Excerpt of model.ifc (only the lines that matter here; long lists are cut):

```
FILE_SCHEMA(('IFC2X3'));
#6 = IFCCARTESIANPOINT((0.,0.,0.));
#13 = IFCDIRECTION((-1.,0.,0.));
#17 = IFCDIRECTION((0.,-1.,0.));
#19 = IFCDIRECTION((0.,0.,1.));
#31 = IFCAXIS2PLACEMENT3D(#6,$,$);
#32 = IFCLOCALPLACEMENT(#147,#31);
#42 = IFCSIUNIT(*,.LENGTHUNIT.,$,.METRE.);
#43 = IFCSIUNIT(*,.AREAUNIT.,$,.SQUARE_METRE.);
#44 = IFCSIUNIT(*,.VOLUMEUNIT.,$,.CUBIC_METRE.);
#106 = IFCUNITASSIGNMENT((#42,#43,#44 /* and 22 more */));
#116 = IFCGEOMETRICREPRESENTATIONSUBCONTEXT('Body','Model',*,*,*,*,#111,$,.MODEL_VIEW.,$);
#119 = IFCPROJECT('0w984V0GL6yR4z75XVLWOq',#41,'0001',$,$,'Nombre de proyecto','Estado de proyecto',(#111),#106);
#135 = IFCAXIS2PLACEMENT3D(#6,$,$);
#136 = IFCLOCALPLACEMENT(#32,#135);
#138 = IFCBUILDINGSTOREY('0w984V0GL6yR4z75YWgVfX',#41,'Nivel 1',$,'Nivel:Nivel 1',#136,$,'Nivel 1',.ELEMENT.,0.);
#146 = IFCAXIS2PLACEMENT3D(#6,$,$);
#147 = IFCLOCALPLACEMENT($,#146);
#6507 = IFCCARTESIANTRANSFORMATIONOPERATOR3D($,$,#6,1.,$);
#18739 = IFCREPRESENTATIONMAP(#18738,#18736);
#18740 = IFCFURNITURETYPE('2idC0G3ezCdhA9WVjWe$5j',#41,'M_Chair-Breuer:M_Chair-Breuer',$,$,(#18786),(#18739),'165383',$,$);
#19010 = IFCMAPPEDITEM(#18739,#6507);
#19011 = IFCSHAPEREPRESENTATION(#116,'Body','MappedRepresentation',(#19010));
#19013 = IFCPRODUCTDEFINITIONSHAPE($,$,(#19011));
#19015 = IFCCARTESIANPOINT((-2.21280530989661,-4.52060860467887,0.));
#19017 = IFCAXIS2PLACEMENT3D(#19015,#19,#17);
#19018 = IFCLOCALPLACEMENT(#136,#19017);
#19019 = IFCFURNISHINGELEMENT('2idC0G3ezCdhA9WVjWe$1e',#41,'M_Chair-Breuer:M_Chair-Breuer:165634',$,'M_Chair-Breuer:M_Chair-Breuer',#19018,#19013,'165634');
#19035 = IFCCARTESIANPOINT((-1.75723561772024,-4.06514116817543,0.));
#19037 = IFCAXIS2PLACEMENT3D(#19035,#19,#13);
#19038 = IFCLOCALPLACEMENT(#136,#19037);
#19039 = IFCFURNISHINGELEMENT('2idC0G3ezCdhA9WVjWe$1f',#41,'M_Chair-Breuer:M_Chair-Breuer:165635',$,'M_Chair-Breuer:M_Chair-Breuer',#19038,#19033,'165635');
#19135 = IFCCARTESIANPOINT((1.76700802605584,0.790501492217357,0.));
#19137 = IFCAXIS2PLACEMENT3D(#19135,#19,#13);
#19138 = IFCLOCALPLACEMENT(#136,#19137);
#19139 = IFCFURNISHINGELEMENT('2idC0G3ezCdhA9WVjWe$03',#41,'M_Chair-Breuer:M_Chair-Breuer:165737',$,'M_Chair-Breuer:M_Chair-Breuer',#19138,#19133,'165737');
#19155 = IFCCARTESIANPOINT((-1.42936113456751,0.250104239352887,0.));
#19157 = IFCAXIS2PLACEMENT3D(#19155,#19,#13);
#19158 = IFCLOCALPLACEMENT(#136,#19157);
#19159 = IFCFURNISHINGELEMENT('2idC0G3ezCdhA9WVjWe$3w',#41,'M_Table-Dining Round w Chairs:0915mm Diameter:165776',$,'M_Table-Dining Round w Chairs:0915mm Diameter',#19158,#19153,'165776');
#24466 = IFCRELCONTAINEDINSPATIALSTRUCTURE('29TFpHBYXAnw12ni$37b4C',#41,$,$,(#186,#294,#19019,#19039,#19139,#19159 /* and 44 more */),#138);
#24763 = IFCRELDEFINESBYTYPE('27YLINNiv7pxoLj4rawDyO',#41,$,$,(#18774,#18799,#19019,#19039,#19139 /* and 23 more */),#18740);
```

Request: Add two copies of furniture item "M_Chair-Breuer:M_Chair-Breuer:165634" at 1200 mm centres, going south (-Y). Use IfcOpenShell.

```python
import numpy as np
import ifcopenshell
import ifcopenshell.api.geometry
import ifcopenshell.api.root
import ifcopenshell.util.element
import ifcopenshell.util.placement

model = ifcopenshell.open("model.ifc")


def reuse_history(source, copy):
    """copy_class also copies each property set's owner history, people and application; keep the originals."""
    for rel in copy.IsDefinedBy:
        if rel.is_a("IfcRelDefinesByProperties") and (history := rel.RelatingPropertyDefinition.OwnerHistory):
            rel.RelatingPropertyDefinition.OwnerHistory = source.OwnerHistory
            ifcopenshell.util.element.remove_deep2(model, history)


source = model.by_guid("2idC0G3ezCdhA9WVjWe$1e")
base = ifcopenshell.util.placement.get_local_placement(source.ObjectPlacement)
step = np.array([0.0, -1.0, 0.0]) * 1.2

for i in range(1, 3):
    copy = ifcopenshell.api.root.copy_class(model, product=source)
    copy.Representation = ifcopenshell.util.element.copy_deep(
        model, source.Representation, exclude=["IfcGeometricRepresentationContext", "IfcRepresentationMap"]
    )
    copy.Name = "M_Chair-Breuer:M_Chair-Breuer"
    copy.Tag = None
    reuse_history(source, copy)
    matrix = base.copy()
    matrix[:3, 3] += i * step
    print("added at", matrix[:3, 3].round(3) + 0.0)
    ifcopenshell.api.geometry.edit_object_placement(model, product=copy, matrix=matrix, is_si=False)

model.write("model_rev.ifc")
```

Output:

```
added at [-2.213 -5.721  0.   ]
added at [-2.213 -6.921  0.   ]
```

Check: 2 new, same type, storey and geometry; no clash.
